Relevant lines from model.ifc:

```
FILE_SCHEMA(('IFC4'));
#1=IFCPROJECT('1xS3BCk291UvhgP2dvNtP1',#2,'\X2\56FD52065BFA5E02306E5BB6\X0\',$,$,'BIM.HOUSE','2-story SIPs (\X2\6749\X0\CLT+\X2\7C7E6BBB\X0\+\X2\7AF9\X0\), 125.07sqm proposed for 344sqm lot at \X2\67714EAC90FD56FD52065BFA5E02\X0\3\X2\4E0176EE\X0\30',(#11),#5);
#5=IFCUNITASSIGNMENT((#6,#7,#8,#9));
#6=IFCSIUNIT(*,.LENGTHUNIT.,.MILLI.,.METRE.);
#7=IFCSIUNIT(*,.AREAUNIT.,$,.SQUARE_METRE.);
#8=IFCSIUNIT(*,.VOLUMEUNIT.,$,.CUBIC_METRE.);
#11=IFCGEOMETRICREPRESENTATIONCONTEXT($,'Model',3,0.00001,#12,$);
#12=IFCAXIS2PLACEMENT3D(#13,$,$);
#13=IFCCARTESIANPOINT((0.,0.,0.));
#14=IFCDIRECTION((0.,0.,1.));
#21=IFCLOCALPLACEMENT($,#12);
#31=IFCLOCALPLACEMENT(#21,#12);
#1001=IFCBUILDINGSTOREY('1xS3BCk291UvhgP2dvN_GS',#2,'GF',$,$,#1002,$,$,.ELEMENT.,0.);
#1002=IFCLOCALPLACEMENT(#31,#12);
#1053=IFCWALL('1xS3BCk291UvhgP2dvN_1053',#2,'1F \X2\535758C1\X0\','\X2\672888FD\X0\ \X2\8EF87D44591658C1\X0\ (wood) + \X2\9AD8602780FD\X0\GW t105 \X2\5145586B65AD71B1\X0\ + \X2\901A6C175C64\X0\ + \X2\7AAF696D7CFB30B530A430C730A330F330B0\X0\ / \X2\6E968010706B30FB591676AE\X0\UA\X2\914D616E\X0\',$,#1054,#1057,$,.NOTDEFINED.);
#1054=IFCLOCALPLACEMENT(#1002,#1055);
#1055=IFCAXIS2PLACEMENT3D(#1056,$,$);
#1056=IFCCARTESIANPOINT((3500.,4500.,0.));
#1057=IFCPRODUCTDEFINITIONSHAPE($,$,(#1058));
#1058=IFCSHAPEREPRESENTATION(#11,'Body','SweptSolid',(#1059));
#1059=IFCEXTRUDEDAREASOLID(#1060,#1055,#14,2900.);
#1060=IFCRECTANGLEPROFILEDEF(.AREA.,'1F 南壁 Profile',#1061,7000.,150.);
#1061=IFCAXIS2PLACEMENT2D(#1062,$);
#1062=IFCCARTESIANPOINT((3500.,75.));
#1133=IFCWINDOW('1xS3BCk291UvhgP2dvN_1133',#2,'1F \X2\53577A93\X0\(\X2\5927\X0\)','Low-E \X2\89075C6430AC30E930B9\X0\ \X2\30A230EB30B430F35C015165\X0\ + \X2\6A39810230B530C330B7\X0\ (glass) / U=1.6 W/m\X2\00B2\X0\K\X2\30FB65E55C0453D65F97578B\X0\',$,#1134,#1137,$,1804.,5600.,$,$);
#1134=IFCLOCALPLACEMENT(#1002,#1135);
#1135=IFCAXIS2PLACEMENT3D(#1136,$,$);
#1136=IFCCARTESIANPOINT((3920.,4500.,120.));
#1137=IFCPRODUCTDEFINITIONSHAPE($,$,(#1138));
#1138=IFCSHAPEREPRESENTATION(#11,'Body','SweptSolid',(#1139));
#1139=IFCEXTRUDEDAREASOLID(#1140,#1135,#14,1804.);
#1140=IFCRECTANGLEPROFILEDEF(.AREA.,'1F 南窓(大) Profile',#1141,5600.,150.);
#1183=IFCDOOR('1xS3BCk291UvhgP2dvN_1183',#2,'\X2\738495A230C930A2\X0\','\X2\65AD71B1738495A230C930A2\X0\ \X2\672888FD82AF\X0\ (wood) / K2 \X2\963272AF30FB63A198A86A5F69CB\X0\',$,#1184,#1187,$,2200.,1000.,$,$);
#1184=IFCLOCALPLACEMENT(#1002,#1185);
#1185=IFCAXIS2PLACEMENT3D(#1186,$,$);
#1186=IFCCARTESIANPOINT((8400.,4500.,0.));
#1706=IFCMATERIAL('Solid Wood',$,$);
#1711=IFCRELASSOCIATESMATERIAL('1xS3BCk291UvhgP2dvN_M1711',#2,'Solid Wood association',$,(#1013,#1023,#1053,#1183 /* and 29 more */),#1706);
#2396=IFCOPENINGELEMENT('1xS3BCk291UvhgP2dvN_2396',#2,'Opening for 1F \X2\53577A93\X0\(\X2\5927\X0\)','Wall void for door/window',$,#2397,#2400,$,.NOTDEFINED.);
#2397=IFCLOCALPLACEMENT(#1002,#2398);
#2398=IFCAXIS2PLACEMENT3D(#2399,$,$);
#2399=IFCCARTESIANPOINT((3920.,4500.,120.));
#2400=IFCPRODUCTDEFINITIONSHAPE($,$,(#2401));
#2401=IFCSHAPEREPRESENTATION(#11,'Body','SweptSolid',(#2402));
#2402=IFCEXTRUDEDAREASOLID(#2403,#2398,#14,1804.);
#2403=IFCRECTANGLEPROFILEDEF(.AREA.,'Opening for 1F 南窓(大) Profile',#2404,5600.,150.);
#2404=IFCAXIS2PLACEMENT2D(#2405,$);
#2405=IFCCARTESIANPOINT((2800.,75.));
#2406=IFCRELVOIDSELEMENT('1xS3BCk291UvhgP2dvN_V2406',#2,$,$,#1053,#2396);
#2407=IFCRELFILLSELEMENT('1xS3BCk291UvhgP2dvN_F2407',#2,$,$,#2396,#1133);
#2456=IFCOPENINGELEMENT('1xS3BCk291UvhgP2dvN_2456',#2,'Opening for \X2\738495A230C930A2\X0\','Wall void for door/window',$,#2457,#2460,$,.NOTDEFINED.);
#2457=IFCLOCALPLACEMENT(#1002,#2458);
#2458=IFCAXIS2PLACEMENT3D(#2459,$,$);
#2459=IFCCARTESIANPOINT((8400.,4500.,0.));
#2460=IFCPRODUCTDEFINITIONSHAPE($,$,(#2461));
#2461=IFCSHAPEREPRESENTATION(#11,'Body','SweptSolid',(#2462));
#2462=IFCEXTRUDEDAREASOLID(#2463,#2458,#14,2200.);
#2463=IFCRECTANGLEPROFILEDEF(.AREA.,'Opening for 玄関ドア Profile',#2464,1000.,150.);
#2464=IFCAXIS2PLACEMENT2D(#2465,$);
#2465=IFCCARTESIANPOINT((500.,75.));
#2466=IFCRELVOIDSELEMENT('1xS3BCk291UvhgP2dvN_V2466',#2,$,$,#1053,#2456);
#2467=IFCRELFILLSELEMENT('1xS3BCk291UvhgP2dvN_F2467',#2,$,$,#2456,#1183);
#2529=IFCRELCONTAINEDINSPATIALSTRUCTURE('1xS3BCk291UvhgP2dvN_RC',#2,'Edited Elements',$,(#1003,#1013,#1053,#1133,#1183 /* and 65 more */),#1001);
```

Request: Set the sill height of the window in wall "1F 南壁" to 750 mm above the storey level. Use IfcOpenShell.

```python
import numpy as np
import ifcopenshell
import ifcopenshell.api.geometry
import ifcopenshell.geom
import ifcopenshell.util.element
import ifcopenshell.util.placement
import ifcopenshell.util.shape
import ifcopenshell.util.unit

model = ifcopenshell.open("model.ifc")
unit_scale = ifcopenshell.util.unit.calculate_unit_scale(model)

window = model.by_guid("1xS3BCk291UvhgP2dvN_1133")
opening = window.FillsVoids[0].RelatingOpeningElement
storey = ifcopenshell.util.element.get_container(window, ifc_class="IfcBuildingStorey")
level = ifcopenshell.util.placement.get_local_placement(storey.ObjectPlacement)[2, 3]

# The opening's origin need not be at the sill, so measure its lowest point.
shape = ifcopenshell.geom.create_shape(ifcopenshell.geom.settings(), opening)
bottom = ifcopenshell.util.shape.get_shape_bottom_elevation(shape, shape.geometry) / unit_scale
dz = level + 0.75 / unit_scale - bottom

shift = np.array([0.0, 0.0, dz])
# The window is not placed relative to its opening, so move both.
for product in (opening, window):
    matrix = ifcopenshell.util.placement.get_local_placement(product.ObjectPlacement)
    matrix[:3, 3] += shift
    ifcopenshell.api.geometry.edit_object_placement(model, product=product, matrix=matrix, is_si=False)

print(f"moved by {dz * unit_scale:+.3f} m")

model.write("model_rev.ifc")
```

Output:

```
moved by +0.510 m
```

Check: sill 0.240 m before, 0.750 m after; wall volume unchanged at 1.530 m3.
